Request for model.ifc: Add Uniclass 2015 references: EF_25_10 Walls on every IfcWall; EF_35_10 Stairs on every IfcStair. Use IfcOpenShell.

First a look at what the model holds.

```python
import ifcopenshell

model = ifcopenshell.open("model.ifc")
print(model.schema)
print("classifications:", [c.Name for c in model.by_type("IfcClassification")])
for ifc_class in ("IfcDoor", "IfcRoof", "IfcStair", "IfcWall", "IfcWindow"):
    print(ifc_class, len(model.by_type(ifc_class)))
```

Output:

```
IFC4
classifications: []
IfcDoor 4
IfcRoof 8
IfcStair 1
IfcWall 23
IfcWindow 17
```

```python
import ifcopenshell
import ifcopenshell.api.classification

model = ifcopenshell.open("model.ifc")

system = ifcopenshell.api.classification.add_classification(model, classification="Uniclass 2015")

codes = {
    "IfcWall": ("EF_25_10", "Walls"),
    "IfcStair": ("EF_35_10", "Stairs"),
}
for ifc_class, (code, name) in codes.items():
    products = model.by_type(ifc_class)
    ifcopenshell.api.classification.add_reference(
        model, products=products, classification=system, identification=code, name=name
    )
    print(code, len(products))

model.write("model_v2.ifc")
```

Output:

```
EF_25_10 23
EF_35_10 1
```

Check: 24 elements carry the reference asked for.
